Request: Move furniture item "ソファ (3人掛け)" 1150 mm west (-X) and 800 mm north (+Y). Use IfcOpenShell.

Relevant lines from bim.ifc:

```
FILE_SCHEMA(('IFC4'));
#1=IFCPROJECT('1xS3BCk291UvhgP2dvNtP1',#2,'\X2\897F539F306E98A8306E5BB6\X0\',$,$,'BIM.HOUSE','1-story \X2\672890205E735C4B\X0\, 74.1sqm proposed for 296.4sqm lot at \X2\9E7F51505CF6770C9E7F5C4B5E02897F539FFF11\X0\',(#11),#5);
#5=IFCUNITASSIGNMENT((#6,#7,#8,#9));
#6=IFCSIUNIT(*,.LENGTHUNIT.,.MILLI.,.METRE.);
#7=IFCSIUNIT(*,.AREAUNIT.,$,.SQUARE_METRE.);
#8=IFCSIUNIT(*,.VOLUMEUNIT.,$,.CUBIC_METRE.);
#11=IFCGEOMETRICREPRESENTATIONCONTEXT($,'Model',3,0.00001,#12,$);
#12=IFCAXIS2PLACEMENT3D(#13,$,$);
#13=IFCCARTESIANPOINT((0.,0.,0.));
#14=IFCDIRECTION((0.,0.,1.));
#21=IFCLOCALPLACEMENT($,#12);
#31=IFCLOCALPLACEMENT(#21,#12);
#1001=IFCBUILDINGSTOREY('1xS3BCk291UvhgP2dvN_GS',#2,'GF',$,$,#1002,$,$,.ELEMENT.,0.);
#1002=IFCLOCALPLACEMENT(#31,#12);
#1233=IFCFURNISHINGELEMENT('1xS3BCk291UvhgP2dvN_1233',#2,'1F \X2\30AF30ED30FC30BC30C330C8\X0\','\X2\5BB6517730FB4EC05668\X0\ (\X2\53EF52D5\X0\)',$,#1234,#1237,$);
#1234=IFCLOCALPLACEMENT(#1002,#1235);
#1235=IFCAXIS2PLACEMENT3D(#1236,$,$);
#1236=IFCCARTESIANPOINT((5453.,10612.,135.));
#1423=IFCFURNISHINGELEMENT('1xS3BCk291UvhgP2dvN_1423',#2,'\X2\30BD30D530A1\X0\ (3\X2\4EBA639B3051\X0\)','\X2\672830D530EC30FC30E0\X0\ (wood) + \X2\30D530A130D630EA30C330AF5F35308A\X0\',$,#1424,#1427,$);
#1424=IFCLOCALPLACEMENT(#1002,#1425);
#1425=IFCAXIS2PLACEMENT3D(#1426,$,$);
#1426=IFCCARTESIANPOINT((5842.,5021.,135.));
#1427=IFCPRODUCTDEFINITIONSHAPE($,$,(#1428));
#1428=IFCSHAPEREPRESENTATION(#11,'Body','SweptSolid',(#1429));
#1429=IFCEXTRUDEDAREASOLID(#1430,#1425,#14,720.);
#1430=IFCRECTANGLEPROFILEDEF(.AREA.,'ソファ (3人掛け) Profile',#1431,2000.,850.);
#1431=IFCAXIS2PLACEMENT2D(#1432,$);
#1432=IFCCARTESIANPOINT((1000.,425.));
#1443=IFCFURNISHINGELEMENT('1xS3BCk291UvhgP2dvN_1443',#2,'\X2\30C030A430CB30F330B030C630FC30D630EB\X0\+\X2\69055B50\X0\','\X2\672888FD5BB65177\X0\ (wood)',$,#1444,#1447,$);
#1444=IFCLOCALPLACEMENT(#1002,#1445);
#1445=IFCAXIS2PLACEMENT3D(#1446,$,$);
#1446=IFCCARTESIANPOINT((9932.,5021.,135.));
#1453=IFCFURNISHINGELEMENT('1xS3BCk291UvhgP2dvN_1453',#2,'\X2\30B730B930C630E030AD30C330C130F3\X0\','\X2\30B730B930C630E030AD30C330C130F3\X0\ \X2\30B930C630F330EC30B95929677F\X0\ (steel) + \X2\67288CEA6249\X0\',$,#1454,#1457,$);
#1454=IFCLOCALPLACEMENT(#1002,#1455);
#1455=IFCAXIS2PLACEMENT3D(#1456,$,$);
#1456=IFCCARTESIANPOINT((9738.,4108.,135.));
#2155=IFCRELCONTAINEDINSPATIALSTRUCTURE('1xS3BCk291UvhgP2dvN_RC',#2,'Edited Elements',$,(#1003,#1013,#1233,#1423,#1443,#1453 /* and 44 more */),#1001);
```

```python
import ifcopenshell
import ifcopenshell.api.geometry
import ifcopenshell.util.placement

model = ifcopenshell.open("bim.ifc")

item = model.by_guid("1xS3BCk291UvhgP2dvN_1423")
matrix = ifcopenshell.util.placement.get_local_placement(item.ObjectPlacement)
matrix[0, 3] -= 1150.0
matrix[1, 3] += 800.0
ifcopenshell.api.geometry.edit_object_placement(model, product=item, matrix=matrix, is_si=False)

print(ifcopenshell.util.placement.get_local_placement(item.ObjectPlacement).round(3) + 0.0)

model.write("bim_v2.ifc")
```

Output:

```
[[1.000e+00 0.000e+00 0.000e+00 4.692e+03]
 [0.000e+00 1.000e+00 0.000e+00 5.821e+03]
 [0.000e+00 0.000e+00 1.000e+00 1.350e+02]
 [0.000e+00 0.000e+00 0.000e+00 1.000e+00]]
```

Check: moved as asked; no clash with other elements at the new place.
